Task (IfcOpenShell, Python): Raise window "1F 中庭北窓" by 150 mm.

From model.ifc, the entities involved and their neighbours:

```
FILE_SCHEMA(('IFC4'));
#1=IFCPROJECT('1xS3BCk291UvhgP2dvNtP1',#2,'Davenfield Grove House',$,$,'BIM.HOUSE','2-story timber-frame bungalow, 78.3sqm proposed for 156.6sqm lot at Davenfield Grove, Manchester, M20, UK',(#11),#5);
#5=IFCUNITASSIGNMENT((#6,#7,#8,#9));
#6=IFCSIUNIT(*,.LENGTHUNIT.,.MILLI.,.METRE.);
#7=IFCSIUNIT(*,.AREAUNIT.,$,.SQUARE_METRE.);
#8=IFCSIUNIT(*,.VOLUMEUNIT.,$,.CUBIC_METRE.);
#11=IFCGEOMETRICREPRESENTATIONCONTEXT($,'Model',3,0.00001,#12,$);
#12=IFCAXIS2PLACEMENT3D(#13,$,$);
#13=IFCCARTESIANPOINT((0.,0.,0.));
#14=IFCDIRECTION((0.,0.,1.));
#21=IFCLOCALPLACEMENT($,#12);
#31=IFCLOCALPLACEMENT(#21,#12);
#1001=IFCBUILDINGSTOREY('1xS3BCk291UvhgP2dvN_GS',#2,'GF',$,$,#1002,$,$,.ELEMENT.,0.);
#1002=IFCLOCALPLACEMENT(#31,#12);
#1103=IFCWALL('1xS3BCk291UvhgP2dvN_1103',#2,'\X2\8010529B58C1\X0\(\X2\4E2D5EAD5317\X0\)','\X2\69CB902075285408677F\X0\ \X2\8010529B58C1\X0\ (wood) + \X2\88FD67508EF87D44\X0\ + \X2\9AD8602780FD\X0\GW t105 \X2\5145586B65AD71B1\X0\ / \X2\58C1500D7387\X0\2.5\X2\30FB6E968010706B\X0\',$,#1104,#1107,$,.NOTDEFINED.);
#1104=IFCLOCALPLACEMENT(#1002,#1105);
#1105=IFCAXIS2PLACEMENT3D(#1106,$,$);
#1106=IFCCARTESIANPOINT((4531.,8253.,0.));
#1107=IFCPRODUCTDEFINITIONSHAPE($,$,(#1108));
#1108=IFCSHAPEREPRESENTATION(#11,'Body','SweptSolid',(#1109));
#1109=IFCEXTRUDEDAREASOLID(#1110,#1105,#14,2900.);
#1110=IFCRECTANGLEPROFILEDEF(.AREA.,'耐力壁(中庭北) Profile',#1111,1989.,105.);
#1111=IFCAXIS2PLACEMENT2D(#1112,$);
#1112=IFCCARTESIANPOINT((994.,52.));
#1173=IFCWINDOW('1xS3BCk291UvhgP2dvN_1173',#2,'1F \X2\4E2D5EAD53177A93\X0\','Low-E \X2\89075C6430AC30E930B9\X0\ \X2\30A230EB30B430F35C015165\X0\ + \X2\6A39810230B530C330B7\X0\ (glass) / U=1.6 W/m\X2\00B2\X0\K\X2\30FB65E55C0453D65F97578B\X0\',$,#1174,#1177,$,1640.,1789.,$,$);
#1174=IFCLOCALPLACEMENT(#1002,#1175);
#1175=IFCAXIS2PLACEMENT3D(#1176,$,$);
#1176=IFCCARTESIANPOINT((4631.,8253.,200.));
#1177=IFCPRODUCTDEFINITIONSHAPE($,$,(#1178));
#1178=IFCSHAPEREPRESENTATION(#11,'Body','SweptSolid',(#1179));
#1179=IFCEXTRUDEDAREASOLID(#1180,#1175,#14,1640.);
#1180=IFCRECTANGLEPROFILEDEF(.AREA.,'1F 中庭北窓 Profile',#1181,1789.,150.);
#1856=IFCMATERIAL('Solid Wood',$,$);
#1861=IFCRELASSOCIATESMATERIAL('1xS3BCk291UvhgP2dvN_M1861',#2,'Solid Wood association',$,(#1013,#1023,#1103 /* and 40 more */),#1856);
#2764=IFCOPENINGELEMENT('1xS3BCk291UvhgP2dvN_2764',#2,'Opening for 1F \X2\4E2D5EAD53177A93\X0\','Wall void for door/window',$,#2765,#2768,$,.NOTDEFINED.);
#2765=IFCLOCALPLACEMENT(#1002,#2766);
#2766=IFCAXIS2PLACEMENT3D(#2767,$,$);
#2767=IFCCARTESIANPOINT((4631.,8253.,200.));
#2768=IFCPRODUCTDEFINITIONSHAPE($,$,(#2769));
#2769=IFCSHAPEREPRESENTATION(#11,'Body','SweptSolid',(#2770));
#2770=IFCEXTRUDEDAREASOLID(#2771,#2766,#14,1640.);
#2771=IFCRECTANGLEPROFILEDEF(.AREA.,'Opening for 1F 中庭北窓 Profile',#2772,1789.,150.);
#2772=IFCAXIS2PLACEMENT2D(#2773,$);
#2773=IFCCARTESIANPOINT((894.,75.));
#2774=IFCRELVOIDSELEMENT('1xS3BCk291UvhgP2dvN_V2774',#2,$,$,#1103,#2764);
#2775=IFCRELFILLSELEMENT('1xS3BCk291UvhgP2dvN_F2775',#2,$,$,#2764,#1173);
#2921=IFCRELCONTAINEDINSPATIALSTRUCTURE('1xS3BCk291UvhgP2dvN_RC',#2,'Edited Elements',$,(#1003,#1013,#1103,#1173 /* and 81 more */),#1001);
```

```python
import numpy as np
import ifcopenshell
import ifcopenshell.api.geometry
import ifcopenshell.util.placement
import ifcopenshell.util.unit

model = ifcopenshell.open("model.ifc")
unit_scale = ifcopenshell.util.unit.calculate_unit_scale(model)

window = model.by_id(1173)
opening = window.FillsVoids[0].RelatingOpeningElement
dz = 0.15 / unit_scale

shift = np.array([0.0, 0.0, dz])
# The window is not placed relative to its opening, so move both.
for product in (opening, window):
    matrix = ifcopenshell.util.placement.get_local_placement(product.ObjectPlacement)
    matrix[:3, 3] += shift
    ifcopenshell.api.geometry.edit_object_placement(model, product=product, matrix=matrix, is_si=False)

print(f"moved by {dz * unit_scale:+.3f} m")

model.write("model-out.ifc")
```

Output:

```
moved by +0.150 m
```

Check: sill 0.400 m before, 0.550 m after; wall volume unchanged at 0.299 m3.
